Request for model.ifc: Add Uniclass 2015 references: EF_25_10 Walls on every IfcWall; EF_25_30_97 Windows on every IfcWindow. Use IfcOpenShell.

First a look at what the model holds.

```python
import ifcopenshell

model = ifcopenshell.open("model.ifc")
print(model.schema)
print("classifications:", [c.Name for c in model.by_type("IfcClassification")])
for ifc_class in ("IfcDoor", "IfcRoof", "IfcStair", "IfcWall", "IfcWindow"):
    print(ifc_class, len(model.by_type(ifc_class)))
```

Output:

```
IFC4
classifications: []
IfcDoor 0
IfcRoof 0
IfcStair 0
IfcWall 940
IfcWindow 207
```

```python
import ifcopenshell
import ifcopenshell.api.classification

model = ifcopenshell.open("model.ifc")

system = ifcopenshell.api.classification.add_classification(model, classification="Uniclass 2015")

codes = {
    "IfcWall": ("EF_25_10", "Walls"),
    "IfcWindow": ("EF_25_30_97", "Windows"),
}
for ifc_class, (code, name) in codes.items():
    products = model.by_type(ifc_class)
    ifcopenshell.api.classification.add_reference(
        model, products=products, classification=system, identification=code, name=name
    )
    print(code, len(products))

model.write("model_edited.ifc")
```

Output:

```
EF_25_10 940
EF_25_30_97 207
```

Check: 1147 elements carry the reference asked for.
